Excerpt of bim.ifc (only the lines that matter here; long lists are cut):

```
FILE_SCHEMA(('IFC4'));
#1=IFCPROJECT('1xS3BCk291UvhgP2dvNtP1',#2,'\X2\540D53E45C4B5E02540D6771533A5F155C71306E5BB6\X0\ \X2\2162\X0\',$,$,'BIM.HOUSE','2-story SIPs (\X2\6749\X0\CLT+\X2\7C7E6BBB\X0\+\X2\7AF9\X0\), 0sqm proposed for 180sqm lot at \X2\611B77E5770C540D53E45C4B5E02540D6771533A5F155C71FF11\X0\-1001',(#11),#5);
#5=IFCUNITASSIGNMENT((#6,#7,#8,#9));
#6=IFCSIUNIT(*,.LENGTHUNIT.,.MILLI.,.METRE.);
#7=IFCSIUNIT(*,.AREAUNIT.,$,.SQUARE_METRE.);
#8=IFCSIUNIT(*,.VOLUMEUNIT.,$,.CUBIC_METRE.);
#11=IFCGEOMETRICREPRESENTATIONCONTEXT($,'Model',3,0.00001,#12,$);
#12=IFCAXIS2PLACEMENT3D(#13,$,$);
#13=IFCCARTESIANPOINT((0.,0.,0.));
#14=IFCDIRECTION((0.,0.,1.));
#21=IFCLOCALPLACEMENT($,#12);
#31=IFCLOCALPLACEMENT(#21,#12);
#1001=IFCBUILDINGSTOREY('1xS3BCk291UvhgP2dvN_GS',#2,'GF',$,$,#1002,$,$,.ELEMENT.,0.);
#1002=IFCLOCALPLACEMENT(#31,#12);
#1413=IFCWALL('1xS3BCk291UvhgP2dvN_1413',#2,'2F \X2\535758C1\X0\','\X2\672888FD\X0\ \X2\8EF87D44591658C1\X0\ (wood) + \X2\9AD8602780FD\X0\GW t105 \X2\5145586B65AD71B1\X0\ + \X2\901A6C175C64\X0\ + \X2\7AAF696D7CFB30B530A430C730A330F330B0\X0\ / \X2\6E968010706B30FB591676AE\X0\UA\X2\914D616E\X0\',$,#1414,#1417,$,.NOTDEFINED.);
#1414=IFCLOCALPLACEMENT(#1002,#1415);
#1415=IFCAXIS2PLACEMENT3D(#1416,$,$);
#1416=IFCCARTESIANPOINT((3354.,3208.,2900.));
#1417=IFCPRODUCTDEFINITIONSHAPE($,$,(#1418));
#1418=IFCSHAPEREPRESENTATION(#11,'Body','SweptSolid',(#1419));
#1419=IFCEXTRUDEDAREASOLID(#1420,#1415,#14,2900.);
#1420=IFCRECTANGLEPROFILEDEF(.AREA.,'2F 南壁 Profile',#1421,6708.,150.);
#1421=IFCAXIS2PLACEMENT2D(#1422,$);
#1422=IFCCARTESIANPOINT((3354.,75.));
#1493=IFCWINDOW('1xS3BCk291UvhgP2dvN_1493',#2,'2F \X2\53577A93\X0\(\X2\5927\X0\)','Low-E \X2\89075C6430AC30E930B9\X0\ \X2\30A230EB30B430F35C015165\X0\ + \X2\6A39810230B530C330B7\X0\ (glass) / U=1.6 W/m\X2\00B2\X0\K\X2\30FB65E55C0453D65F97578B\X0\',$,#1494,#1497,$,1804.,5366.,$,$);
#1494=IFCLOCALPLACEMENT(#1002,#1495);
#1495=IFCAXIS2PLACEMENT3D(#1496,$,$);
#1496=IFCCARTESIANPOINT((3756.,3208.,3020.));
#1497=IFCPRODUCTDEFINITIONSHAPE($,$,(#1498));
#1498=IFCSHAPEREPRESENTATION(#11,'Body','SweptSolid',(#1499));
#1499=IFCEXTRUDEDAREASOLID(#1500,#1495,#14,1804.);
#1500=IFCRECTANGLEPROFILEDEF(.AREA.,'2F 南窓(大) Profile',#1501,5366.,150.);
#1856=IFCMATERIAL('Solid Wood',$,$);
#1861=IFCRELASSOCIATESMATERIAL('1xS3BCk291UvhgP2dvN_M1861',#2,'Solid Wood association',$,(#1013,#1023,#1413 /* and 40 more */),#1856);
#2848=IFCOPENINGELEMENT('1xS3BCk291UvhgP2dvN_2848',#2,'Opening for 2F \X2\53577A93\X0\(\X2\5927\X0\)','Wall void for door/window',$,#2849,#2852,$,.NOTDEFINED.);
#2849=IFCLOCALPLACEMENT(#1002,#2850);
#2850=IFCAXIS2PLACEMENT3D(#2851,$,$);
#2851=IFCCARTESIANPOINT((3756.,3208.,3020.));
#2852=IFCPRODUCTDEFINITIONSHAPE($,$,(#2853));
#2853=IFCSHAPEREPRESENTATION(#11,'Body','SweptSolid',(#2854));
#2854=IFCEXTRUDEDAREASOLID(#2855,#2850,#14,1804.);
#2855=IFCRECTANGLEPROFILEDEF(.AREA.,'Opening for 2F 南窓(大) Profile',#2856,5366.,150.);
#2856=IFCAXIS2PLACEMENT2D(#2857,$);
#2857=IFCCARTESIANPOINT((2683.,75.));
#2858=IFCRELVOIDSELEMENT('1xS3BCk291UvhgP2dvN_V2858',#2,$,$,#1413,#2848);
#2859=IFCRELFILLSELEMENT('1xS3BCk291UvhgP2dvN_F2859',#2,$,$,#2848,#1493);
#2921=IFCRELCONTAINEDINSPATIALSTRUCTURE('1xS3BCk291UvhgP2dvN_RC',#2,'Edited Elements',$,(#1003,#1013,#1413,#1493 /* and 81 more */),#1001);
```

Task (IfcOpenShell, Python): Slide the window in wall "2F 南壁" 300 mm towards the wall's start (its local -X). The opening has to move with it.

```python
import ifcopenshell
import ifcopenshell.api.geometry
import ifcopenshell.util.placement
import ifcopenshell.util.unit

model = ifcopenshell.open("bim.ifc")
unit_scale = ifcopenshell.util.unit.calculate_unit_scale(model)

window = model.by_guid("1xS3BCk291UvhgP2dvN_1493")
opening = window.FillsVoids[0].RelatingOpeningElement
wall = opening.VoidsElements[0].RelatingBuildingElement

wall_matrix = ifcopenshell.util.placement.get_local_placement(wall.ObjectPlacement)
shift = wall_matrix[:3, 0] * -0.3 / unit_scale
before = ifcopenshell.util.placement.get_local_placement(window.ObjectPlacement)[:3, 3].copy()

# The window is not placed relative to its opening, so move both.
for product in (opening, window):
    matrix = ifcopenshell.util.placement.get_local_placement(product.ObjectPlacement)
    matrix[:3, 3] += shift
    ifcopenshell.api.geometry.edit_object_placement(model, product=product, matrix=matrix, is_si=False)

after = ifcopenshell.util.placement.get_local_placement(window.ObjectPlacement)[:3, 3]
print("window moved by", (after - before).round(3) + 0.0)

model.write("bim-out.ifc")
```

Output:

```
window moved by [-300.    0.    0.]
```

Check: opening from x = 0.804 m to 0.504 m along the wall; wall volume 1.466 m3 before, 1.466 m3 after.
